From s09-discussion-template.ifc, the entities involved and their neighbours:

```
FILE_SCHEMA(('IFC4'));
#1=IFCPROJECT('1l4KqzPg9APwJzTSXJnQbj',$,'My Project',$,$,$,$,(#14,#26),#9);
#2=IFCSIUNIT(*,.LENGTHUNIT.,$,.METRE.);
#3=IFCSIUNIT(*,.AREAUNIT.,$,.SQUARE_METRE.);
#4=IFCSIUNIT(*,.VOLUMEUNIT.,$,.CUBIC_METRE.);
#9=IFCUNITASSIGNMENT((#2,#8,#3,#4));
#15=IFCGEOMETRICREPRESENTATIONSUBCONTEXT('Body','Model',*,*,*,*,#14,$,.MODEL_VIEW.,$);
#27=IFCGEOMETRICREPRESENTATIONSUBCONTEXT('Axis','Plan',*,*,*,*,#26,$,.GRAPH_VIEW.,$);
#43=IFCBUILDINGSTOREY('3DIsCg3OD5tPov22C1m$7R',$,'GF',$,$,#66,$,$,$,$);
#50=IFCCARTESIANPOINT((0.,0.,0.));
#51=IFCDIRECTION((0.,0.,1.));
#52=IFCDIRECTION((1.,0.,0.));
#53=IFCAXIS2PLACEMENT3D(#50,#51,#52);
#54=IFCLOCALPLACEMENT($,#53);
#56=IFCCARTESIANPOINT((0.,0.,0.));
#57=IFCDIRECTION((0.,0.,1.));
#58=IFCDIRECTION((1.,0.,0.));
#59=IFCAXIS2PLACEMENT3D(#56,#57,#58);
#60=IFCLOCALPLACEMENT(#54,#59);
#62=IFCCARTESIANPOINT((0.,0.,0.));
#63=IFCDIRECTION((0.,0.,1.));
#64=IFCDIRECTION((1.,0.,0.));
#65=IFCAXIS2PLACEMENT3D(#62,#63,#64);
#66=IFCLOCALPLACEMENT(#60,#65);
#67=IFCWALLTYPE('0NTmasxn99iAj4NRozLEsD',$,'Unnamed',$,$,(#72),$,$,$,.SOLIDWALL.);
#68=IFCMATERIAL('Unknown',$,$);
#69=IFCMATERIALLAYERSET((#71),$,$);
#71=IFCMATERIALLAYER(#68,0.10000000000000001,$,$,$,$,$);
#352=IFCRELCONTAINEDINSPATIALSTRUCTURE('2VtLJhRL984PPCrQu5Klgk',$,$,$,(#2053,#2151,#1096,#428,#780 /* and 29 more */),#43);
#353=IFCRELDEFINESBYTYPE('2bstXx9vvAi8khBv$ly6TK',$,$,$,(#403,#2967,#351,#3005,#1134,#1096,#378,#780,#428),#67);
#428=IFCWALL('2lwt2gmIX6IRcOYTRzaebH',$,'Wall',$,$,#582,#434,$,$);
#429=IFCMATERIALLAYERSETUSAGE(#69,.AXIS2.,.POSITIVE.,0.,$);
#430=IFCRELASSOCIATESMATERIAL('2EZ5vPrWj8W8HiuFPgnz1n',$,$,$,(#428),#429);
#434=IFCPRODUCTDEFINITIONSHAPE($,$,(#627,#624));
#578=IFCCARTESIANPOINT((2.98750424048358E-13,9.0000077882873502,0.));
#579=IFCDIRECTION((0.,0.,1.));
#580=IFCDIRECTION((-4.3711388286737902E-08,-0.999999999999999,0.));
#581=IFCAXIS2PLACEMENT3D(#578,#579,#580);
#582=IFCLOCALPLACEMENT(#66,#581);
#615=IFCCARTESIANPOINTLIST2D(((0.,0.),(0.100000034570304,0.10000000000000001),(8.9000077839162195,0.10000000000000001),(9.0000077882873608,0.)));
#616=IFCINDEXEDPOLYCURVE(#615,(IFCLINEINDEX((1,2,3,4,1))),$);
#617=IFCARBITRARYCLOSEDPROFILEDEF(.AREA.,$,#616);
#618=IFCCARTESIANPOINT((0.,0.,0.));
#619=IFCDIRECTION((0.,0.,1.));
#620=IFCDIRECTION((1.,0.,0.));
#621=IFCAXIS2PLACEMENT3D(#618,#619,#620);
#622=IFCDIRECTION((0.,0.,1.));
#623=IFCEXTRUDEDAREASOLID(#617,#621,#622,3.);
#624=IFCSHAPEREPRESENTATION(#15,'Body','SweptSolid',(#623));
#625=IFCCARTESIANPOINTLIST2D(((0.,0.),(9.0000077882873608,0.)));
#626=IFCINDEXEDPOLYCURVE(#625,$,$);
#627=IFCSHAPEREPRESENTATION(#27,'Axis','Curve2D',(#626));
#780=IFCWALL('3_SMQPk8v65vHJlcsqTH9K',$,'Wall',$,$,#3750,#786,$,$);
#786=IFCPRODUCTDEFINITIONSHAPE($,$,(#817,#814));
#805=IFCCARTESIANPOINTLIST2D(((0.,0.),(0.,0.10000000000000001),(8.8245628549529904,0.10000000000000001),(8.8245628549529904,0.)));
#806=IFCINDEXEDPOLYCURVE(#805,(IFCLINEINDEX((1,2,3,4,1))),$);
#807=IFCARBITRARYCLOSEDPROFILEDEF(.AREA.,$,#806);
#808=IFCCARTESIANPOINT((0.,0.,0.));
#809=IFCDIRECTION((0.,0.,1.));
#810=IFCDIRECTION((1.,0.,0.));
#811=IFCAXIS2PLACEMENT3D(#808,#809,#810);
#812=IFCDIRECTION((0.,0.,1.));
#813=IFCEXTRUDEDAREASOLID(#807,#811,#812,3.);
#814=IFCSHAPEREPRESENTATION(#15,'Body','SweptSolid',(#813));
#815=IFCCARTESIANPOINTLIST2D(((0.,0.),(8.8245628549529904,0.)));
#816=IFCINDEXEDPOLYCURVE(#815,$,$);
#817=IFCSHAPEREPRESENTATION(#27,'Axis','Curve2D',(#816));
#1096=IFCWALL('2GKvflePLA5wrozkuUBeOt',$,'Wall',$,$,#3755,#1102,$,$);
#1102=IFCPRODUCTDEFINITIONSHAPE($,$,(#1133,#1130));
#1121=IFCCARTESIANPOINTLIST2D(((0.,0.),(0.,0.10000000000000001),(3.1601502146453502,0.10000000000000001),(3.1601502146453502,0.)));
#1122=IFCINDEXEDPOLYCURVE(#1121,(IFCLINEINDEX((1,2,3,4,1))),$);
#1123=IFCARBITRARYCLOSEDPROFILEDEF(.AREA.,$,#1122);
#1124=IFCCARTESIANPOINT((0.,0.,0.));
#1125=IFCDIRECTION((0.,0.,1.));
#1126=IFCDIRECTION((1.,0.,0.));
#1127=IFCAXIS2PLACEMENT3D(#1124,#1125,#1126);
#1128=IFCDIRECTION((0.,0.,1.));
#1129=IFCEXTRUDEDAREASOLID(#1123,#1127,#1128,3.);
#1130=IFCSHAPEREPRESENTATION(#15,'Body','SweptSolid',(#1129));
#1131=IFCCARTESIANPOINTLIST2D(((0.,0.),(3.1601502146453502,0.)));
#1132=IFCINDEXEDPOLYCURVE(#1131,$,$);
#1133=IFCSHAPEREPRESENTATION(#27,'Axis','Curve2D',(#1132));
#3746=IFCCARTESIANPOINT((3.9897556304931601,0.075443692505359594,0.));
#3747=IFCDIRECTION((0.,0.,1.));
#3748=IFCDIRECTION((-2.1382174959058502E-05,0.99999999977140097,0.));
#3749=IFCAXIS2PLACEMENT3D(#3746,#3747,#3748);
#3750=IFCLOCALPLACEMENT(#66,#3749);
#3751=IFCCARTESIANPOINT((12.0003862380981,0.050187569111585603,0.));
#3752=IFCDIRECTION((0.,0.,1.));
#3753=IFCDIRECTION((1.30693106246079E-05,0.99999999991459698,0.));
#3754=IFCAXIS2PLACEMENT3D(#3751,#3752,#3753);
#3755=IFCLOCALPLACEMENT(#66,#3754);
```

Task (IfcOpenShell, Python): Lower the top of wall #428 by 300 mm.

```python
import ifcopenshell
import ifcopenshell.geom
import ifcopenshell.util.representation
import ifcopenshell.util.shape

model = ifcopenshell.open("s09-discussion-template.ifc")
settings = ifcopenshell.geom.settings()


def volume(element):
    """Net volume in cubic metres, openings subtracted."""
    shape = ifcopenshell.geom.create_shape(settings, element)
    return ifcopenshell.util.shape.get_volume(shape.geometry)


wall = model.by_guid("2lwt2gmIX6IRcOYTRzaebH")
before = volume(wall)

body = ifcopenshell.util.representation.get_representation(wall, "Model", "Body")
solid = body.Items[0]
old_height = solid.Depth
solid.Depth -= 0.3
after = volume(wall)

print(f"height {old_height:g} -> {solid.Depth:g}, volume {before:.3f} -> {after:.3f} m3")

model.write("s09-discussion-template_edited.ifc")
```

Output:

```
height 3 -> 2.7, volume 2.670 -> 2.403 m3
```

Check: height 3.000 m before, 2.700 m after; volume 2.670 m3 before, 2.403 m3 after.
